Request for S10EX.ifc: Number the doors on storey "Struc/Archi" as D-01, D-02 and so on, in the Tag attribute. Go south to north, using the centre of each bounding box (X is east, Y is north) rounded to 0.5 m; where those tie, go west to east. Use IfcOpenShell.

First a look at what the model holds.

```python
import ifcopenshell
import ifcopenshell.util.element
import ifcopenshell.util.placement

model = ifcopenshell.open("S10EX.ifc")
print(model.schema)
storey = next(s for s in model.by_type("IfcBuildingStorey") if s.Name == "Struc/Archi")
doors = [e for e in ifcopenshell.util.element.get_decomposition(storey) if e.is_a("IfcDoor")]
for e in sorted(doors, key=lambda e: e.id()):
    origin = ifcopenshell.util.placement.get_local_placement(e.ObjectPlacement)[:3, 3]
    print(e.id(), e.Tag, e.Name, origin.round(2) + 0.0, sep=" | ")
```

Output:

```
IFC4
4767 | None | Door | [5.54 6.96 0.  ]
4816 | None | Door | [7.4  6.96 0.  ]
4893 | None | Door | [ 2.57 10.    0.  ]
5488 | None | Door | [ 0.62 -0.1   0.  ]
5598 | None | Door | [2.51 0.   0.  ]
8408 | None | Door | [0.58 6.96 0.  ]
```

```python
import ifcopenshell
import ifcopenshell.geom
import ifcopenshell.util.element
import ifcopenshell.util.shape

model = ifcopenshell.open("S10EX.ifc")
settings = ifcopenshell.geom.settings()
settings.set("use-world-coords", True)


def centre(element):
    shape = ifcopenshell.geom.create_shape(settings, element)
    return ifcopenshell.util.shape.get_bbox_centroid(shape.geometry)


storey = next(s for s in model.by_type("IfcBuildingStorey") if s.Name == "Struc/Archi")
doors = [e for e in ifcopenshell.util.element.get_decomposition(storey) if e.is_a("IfcDoor")]

# Insertion points can sit at a corner or the storey origin, so sort by the geometry (in metres).
centres = {e: centre(e) for e in doors}
doors.sort(key=lambda e: (round(centres[e][1] / 0.5), centres[e][0]))

for i, e in enumerate(doors, start=1):
    number = f"D-{i:02d}"
    e.Tag = number
    print(e.id(), number)

model.write("S10EX_rev.ifc")
```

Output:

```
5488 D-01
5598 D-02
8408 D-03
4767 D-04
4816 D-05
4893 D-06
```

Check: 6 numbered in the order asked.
